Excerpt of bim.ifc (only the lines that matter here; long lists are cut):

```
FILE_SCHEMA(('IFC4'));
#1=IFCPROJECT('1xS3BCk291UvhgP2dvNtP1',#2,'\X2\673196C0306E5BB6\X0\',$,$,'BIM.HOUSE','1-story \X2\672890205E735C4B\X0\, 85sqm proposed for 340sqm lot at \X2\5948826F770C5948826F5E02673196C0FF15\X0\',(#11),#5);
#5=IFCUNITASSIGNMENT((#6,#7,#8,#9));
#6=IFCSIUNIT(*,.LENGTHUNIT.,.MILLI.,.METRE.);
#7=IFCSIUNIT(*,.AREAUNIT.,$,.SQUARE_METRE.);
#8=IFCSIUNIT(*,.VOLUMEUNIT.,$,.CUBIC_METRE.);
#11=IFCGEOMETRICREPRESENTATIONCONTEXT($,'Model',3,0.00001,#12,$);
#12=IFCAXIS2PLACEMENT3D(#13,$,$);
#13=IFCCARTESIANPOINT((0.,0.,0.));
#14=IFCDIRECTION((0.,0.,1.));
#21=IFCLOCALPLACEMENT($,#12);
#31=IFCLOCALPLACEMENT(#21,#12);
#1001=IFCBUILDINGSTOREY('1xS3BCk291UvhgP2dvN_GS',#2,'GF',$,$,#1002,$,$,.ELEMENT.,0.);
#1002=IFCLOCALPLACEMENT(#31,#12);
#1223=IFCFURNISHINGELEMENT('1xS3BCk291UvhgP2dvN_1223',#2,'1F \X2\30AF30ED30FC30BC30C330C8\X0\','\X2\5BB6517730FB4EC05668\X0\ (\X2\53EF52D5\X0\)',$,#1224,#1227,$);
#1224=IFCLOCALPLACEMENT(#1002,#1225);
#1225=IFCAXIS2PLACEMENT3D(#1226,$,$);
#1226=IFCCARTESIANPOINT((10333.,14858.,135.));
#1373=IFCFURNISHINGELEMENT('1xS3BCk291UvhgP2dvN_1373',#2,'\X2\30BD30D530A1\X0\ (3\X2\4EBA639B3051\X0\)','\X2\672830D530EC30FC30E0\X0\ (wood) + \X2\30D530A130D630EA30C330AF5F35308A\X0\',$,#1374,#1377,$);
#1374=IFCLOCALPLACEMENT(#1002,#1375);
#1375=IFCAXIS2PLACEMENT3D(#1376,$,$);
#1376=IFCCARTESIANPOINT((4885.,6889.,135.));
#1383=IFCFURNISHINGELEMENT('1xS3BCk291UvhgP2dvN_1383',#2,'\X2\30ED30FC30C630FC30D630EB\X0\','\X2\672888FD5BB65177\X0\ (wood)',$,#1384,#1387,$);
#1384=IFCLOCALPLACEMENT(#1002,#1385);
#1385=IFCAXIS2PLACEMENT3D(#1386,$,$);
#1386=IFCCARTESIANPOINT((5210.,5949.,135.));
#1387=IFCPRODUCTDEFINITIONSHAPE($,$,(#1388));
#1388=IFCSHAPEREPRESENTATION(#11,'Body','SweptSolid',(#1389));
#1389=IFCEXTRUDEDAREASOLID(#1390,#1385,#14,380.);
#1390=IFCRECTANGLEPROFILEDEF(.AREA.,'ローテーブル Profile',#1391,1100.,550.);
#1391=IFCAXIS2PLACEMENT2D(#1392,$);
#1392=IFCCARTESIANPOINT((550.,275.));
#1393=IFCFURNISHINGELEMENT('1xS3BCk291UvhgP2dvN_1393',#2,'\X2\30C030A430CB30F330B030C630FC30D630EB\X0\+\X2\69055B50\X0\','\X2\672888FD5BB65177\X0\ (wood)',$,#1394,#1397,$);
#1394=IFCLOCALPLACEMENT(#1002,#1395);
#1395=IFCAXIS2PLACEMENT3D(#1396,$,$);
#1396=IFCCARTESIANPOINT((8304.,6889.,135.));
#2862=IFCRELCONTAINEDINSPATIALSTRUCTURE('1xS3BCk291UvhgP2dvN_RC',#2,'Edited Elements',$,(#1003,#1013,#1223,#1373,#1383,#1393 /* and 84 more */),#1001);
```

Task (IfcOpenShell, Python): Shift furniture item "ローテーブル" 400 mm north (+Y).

```python
import ifcopenshell
import ifcopenshell.api.geometry
import ifcopenshell.util.placement

model = ifcopenshell.open("bim.ifc")

item = model.by_guid("1xS3BCk291UvhgP2dvN_1383")
matrix = ifcopenshell.util.placement.get_local_placement(item.ObjectPlacement)
matrix[1, 3] += 400.0
ifcopenshell.api.geometry.edit_object_placement(model, product=item, matrix=matrix, is_si=False)

print(ifcopenshell.util.placement.get_local_placement(item.ObjectPlacement).round(3) + 0.0)

model.write("bim_rev.ifc")
```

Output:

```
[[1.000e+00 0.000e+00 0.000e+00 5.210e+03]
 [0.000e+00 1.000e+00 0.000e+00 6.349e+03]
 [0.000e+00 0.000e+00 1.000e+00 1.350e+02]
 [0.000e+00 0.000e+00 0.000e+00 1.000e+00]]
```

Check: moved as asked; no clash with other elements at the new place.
